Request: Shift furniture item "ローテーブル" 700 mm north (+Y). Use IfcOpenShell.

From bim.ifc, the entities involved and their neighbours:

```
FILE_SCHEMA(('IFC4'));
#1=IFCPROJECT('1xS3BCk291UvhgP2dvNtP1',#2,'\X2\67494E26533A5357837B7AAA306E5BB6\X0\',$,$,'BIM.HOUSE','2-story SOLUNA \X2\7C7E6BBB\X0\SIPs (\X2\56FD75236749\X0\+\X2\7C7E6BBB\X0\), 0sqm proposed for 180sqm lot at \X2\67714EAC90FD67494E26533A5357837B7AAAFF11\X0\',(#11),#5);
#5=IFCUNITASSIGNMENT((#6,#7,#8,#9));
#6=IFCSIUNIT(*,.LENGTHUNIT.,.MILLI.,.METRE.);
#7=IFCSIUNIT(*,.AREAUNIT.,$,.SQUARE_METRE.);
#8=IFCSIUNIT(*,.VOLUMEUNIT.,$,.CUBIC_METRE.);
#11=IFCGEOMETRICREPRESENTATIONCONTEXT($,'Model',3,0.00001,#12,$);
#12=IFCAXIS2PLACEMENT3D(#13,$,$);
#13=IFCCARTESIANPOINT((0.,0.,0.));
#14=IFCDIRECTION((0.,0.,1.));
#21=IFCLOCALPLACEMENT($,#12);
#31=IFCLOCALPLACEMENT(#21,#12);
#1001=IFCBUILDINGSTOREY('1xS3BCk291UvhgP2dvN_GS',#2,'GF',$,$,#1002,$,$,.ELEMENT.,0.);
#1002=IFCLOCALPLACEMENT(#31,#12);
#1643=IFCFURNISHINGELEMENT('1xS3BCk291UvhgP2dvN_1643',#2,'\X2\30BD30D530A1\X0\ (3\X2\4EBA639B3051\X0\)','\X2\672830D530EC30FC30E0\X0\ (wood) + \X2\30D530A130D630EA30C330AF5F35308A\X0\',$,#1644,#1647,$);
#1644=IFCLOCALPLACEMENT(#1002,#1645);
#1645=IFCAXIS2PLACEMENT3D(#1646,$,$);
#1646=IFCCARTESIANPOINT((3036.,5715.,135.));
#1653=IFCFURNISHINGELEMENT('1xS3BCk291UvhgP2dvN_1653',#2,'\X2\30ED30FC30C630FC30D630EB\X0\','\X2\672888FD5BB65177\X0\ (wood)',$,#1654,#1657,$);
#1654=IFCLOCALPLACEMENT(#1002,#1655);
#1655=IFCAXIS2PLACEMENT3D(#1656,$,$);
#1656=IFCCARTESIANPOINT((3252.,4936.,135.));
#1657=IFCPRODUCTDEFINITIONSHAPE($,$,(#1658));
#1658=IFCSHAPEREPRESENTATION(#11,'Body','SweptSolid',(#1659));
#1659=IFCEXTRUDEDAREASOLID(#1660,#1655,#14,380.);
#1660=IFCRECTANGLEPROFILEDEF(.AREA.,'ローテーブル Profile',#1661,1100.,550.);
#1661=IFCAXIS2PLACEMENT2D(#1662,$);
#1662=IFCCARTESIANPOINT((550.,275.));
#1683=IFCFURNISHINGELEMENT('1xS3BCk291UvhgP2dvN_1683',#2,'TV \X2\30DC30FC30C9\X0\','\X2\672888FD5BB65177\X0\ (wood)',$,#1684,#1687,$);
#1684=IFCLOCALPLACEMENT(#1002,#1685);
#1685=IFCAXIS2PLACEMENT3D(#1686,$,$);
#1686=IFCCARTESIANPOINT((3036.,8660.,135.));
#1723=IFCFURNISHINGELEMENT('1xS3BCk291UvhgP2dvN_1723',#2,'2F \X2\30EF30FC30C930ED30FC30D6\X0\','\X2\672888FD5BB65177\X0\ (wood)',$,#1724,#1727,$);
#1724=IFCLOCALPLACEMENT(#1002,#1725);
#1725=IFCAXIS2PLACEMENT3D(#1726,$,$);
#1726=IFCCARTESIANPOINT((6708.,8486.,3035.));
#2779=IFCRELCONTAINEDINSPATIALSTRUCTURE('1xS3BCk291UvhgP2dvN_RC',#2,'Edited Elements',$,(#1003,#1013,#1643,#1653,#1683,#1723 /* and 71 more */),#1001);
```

```python
import ifcopenshell
import ifcopenshell.api.geometry
import ifcopenshell.util.placement

model = ifcopenshell.open("bim.ifc")

item = model.by_guid("1xS3BCk291UvhgP2dvN_1653")
matrix = ifcopenshell.util.placement.get_local_placement(item.ObjectPlacement)
matrix[1, 3] += 700.0
ifcopenshell.api.geometry.edit_object_placement(model, product=item, matrix=matrix, is_si=False)

print(ifcopenshell.util.placement.get_local_placement(item.ObjectPlacement).round(3) + 0.0)

model.write("bim_rev.ifc")
```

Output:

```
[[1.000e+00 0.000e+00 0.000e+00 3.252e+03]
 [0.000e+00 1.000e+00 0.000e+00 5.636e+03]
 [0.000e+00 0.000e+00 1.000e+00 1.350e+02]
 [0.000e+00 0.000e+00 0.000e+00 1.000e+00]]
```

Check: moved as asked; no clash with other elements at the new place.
